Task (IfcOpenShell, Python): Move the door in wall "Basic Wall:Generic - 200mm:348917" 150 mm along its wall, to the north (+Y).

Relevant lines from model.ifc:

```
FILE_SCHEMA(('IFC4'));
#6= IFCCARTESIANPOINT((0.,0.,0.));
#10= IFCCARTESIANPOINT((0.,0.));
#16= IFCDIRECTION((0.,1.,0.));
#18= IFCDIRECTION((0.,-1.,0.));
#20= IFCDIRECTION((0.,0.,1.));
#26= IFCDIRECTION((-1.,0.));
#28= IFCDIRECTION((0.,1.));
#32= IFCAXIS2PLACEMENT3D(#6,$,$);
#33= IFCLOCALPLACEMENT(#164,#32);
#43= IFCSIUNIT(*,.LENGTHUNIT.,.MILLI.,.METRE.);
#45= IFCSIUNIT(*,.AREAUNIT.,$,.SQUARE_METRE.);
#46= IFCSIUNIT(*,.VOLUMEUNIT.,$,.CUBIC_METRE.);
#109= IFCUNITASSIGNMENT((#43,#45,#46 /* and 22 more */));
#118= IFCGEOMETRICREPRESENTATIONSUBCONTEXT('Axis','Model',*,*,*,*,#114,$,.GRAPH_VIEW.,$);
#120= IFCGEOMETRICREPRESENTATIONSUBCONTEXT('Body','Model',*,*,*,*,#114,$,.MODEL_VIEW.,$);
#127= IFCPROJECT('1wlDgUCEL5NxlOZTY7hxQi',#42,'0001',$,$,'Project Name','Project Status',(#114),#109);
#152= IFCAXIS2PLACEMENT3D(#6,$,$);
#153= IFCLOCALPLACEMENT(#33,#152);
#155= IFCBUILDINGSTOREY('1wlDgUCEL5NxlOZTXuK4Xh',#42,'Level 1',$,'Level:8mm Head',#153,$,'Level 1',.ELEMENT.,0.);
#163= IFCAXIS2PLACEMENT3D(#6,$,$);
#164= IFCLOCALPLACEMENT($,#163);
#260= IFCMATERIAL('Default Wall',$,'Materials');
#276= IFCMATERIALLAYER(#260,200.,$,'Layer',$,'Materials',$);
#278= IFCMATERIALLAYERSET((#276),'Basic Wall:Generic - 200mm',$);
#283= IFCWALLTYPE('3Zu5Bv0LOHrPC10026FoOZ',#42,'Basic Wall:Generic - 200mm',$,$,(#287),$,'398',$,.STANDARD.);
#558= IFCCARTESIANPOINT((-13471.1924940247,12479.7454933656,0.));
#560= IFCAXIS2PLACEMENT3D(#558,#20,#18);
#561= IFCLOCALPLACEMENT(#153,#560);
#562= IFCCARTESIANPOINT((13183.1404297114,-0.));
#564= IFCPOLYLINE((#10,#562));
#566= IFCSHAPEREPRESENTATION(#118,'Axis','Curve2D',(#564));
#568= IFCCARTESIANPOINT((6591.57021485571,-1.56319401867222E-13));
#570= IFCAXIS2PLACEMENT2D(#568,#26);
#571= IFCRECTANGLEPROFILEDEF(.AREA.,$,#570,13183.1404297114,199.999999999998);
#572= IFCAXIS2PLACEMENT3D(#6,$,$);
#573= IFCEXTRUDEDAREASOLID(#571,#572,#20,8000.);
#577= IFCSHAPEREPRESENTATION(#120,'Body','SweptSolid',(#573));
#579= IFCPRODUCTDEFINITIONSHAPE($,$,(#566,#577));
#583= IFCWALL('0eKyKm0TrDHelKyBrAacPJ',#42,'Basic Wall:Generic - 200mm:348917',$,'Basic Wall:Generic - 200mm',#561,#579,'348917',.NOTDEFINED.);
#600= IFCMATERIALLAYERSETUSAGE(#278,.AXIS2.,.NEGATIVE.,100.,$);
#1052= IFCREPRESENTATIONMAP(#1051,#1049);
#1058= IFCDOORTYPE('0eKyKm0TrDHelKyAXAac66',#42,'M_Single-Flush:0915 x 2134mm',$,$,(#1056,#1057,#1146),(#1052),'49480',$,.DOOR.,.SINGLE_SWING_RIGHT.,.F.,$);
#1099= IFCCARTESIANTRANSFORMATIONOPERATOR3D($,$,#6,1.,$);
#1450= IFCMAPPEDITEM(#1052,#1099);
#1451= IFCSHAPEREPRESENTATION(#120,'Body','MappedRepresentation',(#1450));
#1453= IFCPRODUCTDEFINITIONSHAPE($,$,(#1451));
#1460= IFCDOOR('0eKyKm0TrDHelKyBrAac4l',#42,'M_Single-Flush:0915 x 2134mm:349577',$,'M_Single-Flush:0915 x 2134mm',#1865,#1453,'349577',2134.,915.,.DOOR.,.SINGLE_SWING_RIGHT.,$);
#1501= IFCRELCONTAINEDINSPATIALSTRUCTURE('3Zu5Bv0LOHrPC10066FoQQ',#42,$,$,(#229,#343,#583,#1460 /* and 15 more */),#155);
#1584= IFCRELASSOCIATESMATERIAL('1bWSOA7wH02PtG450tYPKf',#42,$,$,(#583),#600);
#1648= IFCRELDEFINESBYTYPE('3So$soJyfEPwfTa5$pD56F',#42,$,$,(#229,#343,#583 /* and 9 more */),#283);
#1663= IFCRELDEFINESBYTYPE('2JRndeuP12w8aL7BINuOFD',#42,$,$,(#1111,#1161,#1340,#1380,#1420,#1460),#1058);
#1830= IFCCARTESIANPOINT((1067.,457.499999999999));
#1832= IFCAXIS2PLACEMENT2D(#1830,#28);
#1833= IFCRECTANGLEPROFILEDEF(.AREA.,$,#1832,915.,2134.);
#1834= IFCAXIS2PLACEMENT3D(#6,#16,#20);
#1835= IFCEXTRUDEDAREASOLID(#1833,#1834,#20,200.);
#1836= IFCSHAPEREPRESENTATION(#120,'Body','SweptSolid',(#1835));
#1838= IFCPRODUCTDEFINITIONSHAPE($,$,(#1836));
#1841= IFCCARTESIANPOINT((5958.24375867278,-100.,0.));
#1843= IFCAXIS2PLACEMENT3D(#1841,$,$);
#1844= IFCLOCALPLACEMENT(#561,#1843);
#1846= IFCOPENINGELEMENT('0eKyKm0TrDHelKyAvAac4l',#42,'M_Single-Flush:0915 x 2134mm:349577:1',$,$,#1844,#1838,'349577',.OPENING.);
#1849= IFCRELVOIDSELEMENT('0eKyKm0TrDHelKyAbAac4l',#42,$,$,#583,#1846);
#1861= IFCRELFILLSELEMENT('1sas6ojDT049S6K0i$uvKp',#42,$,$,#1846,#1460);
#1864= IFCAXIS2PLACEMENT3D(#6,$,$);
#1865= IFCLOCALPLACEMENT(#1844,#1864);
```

```python
import ifcopenshell
import ifcopenshell.api.geometry
import ifcopenshell.util.placement
import ifcopenshell.util.unit

model = ifcopenshell.open("model.ifc")
unit_scale = ifcopenshell.util.unit.calculate_unit_scale(model)

door = model.by_id(1460)
opening = door.FillsVoids[0].RelatingOpeningElement
wall = opening.VoidsElements[0].RelatingBuildingElement

wall_matrix = ifcopenshell.util.placement.get_local_placement(wall.ObjectPlacement)
shift = wall_matrix[:3, 0] * -0.15 / unit_scale
before = ifcopenshell.util.placement.get_local_placement(door.ObjectPlacement)[:3, 3].copy()

# The door is placed relative to its opening, so it follows when the opening moves.
matrix = ifcopenshell.util.placement.get_local_placement(opening.ObjectPlacement)
matrix[:3, 3] += shift
ifcopenshell.api.geometry.edit_object_placement(
    model, product=opening, matrix=matrix, is_si=False, should_transform_children=True
)

after = ifcopenshell.util.placement.get_local_placement(door.ObjectPlacement)[:3, 3]
print("door moved by", (after - before).round(3) + 0.0)

model.write("model_v2.ifc")
```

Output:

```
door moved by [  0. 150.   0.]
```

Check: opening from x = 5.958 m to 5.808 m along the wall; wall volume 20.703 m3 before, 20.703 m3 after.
